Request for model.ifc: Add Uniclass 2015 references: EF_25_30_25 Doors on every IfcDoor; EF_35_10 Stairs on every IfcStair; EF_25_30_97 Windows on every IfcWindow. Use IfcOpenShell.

First a look at what the model holds.

```python
import ifcopenshell

model = ifcopenshell.open("model.ifc")
print(model.schema)
print("classifications:", [c.Name for c in model.by_type("IfcClassification")])
for ifc_class in ("IfcDoor", "IfcRoof", "IfcStair", "IfcWall", "IfcWindow"):
    print(ifc_class, len(model.by_type(ifc_class)))
```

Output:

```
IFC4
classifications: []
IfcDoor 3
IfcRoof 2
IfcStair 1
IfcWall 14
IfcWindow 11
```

```python
import ifcopenshell
import ifcopenshell.api.classification

model = ifcopenshell.open("model.ifc")

system = ifcopenshell.api.classification.add_classification(model, classification="Uniclass 2015")

codes = {
    "IfcDoor": ("EF_25_30_25", "Doors"),
    "IfcStair": ("EF_35_10", "Stairs"),
    "IfcWindow": ("EF_25_30_97", "Windows"),
}
for ifc_class, (code, name) in codes.items():
    products = model.by_type(ifc_class)
    ifcopenshell.api.classification.add_reference(
        model, products=products, classification=system, identification=code, name=name
    )
    print(code, len(products))

model.write("model-out.ifc")
```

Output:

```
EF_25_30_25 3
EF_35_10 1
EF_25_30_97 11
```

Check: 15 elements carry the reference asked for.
